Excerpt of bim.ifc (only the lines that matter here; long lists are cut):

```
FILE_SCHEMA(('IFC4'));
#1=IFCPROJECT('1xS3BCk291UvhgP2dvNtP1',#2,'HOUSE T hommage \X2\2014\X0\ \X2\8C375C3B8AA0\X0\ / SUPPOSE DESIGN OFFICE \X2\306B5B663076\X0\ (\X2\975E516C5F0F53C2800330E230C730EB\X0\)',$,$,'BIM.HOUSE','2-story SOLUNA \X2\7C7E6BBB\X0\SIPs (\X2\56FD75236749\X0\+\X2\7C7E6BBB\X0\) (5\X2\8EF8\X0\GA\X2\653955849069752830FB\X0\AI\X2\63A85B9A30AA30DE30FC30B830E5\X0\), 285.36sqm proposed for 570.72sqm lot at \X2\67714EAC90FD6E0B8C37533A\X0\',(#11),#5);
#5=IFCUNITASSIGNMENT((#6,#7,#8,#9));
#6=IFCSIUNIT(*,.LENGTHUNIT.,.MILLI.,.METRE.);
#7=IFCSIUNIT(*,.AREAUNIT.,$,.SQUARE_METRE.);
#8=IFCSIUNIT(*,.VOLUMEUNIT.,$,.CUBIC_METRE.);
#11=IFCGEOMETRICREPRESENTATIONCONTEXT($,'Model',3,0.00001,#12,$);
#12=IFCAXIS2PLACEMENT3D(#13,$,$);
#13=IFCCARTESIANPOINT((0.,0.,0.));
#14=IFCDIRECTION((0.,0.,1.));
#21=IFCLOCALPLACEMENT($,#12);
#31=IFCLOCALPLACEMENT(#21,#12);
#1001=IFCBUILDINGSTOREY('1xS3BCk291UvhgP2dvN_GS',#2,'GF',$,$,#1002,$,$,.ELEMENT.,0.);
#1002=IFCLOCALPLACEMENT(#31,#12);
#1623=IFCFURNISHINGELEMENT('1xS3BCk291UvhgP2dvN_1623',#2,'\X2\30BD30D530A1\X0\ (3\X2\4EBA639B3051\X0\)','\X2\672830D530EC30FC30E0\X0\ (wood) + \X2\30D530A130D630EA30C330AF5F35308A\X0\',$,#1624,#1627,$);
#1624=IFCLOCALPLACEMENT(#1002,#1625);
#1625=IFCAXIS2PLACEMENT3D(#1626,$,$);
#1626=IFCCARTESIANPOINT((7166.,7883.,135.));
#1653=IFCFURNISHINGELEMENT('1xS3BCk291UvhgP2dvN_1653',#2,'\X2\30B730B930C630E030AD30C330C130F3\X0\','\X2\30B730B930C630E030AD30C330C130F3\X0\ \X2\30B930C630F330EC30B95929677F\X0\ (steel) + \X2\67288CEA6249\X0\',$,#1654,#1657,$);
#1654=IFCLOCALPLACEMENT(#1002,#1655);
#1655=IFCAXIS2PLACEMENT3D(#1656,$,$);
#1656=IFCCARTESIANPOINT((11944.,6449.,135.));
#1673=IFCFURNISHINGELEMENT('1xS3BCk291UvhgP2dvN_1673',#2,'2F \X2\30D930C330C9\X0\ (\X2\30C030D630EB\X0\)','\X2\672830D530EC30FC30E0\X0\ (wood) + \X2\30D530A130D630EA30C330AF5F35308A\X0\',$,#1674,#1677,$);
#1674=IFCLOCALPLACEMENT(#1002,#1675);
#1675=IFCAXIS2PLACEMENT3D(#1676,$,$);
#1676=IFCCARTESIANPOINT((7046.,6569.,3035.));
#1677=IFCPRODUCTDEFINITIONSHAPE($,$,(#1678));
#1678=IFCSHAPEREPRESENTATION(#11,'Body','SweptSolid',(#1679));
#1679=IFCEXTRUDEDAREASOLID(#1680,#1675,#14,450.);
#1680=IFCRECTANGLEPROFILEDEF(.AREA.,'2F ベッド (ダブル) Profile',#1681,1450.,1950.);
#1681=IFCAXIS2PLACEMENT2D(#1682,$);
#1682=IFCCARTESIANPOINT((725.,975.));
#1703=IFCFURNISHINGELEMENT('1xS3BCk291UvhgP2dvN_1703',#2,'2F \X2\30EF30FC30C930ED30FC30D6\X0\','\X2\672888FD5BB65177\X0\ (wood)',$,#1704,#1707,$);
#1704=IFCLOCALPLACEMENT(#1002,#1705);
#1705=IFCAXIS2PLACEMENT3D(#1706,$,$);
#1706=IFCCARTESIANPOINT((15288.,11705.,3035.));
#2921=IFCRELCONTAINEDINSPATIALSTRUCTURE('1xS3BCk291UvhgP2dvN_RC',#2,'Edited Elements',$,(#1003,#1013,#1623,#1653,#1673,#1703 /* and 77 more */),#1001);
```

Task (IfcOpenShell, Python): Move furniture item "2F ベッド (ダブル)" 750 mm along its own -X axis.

```python
import ifcopenshell
import ifcopenshell.api.geometry
import ifcopenshell.util.placement
import ifcopenshell.util.unit

model = ifcopenshell.open("bim.ifc")
unit_scale = ifcopenshell.util.unit.calculate_unit_scale(model)

item = model.by_guid("1xS3BCk291UvhgP2dvN_1673")
matrix = ifcopenshell.util.placement.get_local_placement(item.ObjectPlacement)
matrix[:3, 3] -= matrix[:3, 0] * 0.75 / unit_scale
ifcopenshell.api.geometry.edit_object_placement(model, product=item, matrix=matrix, is_si=False)

print(ifcopenshell.util.placement.get_local_placement(item.ObjectPlacement).round(3) + 0.0)

model.write("bim-out.ifc")
```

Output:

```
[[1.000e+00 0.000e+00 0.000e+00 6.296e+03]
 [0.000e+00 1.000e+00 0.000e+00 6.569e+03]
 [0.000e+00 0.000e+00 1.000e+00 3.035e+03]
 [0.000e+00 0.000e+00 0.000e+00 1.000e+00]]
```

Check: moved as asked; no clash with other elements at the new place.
